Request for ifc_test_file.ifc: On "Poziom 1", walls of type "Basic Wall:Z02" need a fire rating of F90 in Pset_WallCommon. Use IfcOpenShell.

First a look at what the model holds.

```python
import ifcopenshell
import ifcopenshell.util.element

model = ifcopenshell.open("ifc_test_file.ifc")
print(model.schema)
storey = next(s for s in model.by_type("IfcBuildingStorey") if s.Name == "Poziom 1")
walls = [e for e in ifcopenshell.util.element.get_decomposition(storey) if e.is_a("IfcWall")]
seen = {}
for e in walls:
    element_type = ifcopenshell.util.element.get_type(e)
    key = (element_type.Name if element_type != e and element_type else None, ifcopenshell.util.element.get_pset(e, "Pset_WallCommon", "FireRating"))
    seen[key] = seen.get(key, 0) + 1
for (name, value), count in sorted(seen.items(), key=str):
    print(count, "x", name, "|", value)
```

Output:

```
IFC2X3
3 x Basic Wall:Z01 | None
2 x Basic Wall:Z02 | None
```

```python
import ifcopenshell
import ifcopenshell.api.pset
import ifcopenshell.util.element

model = ifcopenshell.open("ifc_test_file.ifc")

storey = next(s for s in model.by_type("IfcBuildingStorey") if s.Name == "Poziom 1")
walls = [e for e in ifcopenshell.util.element.get_decomposition(storey) if e.is_a("IfcWall")]

count = 0
for e in walls:
    element_type = ifcopenshell.util.element.get_type(e)
    if element_type in (None, e) or element_type.Name != "Basic Wall:Z02":
        continue
    # add_pset returns the element's existing set when there is one.
    pset = ifcopenshell.api.pset.add_pset(model, product=e, name="Pset_WallCommon")
    ifcopenshell.api.pset.edit_pset(model, pset=pset, properties={"FireRating": "F90"})
    count += 1

print(count, "walls updated")

model.write("ifc_test_file_edited.ifc")
```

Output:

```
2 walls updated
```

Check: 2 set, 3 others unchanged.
